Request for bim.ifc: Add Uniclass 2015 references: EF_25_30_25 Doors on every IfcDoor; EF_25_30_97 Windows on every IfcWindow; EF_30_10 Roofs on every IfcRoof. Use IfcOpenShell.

First a look at what the model holds.

```python
import ifcopenshell

model = ifcopenshell.open("bim.ifc")
print(model.schema)
print("classifications:", [c.Name for c in model.by_type("IfcClassification")])
for ifc_class in ("IfcDoor", "IfcRoof", "IfcStair", "IfcWall", "IfcWindow"):
    print(ifc_class, len(model.by_type(ifc_class)))
```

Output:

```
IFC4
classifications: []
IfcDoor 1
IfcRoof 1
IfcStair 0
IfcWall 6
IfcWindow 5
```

```python
import ifcopenshell
import ifcopenshell.api.classification

model = ifcopenshell.open("bim.ifc")

system = ifcopenshell.api.classification.add_classification(model, classification="Uniclass 2015")

codes = {
    "IfcDoor": ("EF_25_30_25", "Doors"),
    "IfcWindow": ("EF_25_30_97", "Windows"),
    "IfcRoof": ("EF_30_10", "Roofs"),
}
for ifc_class, (code, name) in codes.items():
    products = model.by_type(ifc_class)
    ifcopenshell.api.classification.add_reference(
        model, products=products, classification=system, identification=code, name=name
    )
    print(code, len(products))

model.write("bim_updated.ifc")
```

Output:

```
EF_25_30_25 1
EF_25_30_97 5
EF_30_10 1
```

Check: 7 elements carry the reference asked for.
